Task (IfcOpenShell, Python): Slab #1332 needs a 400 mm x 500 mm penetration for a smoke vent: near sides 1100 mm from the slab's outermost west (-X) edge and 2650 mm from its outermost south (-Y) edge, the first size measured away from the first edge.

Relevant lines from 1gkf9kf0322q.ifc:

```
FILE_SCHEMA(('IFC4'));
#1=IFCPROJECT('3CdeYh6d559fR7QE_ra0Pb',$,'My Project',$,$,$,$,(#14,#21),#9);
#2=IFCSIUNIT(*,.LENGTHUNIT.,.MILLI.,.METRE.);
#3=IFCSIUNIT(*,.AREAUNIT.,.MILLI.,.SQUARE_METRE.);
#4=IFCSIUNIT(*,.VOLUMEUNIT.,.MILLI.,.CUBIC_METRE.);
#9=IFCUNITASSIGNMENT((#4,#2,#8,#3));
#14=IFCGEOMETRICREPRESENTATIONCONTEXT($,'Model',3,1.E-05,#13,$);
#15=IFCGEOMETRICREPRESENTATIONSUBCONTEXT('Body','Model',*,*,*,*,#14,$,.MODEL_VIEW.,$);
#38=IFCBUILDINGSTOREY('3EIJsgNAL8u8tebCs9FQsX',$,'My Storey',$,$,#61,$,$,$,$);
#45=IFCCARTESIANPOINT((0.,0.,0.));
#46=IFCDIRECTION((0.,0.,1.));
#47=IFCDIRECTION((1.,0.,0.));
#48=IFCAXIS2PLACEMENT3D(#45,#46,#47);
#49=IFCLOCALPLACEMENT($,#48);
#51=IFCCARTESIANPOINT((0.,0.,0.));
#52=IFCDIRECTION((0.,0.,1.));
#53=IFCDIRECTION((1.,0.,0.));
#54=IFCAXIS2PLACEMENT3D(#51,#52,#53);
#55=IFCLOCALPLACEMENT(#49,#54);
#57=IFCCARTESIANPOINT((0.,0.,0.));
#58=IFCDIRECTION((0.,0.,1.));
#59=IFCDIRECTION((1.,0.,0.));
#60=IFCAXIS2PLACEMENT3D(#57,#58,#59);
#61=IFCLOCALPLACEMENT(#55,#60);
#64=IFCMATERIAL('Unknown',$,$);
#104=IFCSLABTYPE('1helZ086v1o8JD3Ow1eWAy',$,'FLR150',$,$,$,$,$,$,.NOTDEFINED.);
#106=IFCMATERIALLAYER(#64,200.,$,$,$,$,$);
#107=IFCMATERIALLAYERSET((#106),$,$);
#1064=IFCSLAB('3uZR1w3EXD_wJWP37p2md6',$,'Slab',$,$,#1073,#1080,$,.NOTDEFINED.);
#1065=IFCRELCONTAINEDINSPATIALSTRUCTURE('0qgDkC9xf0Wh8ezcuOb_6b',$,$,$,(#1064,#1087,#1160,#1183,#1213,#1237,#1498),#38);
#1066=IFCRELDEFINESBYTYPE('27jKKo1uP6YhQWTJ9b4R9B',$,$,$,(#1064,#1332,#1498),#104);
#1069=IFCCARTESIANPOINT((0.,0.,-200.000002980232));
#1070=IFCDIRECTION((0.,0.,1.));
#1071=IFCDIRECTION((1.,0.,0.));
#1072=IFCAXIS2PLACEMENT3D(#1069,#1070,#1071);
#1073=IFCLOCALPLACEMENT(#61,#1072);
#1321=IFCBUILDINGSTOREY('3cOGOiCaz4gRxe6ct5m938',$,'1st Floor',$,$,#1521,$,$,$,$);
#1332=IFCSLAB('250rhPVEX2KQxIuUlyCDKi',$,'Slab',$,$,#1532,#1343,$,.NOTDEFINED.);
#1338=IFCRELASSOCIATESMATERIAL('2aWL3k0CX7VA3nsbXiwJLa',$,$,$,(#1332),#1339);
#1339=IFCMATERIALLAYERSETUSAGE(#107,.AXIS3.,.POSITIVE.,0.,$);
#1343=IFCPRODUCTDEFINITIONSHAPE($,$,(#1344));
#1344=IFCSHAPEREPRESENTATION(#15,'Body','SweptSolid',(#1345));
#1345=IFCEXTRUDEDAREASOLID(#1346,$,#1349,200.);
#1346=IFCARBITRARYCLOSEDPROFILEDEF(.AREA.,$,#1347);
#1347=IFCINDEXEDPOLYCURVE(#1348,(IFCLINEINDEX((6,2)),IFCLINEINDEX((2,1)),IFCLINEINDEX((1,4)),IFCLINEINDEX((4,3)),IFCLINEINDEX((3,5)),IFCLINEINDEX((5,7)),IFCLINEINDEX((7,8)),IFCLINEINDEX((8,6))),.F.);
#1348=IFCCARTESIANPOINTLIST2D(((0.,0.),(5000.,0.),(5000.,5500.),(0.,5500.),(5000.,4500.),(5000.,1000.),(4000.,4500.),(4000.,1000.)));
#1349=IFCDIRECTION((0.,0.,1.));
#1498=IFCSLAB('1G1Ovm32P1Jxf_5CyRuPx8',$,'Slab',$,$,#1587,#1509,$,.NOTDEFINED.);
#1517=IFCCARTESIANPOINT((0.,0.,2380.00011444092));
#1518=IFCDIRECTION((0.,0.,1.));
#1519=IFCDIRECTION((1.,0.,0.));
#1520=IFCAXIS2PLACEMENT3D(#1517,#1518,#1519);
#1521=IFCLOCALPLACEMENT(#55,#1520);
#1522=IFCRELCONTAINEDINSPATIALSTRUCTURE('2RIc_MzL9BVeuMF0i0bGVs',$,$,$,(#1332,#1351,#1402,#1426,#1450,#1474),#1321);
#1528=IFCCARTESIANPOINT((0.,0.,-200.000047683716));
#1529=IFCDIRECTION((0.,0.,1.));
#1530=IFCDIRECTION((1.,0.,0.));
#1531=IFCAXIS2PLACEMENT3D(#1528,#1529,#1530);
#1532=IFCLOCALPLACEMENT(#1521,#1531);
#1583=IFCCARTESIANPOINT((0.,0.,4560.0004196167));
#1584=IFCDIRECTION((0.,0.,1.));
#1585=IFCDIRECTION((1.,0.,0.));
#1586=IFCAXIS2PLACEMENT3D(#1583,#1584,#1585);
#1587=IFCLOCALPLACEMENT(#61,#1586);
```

```python
import numpy as np
import ifcopenshell
import ifcopenshell.api.feature
import ifcopenshell.api.geometry
import ifcopenshell.api.root
import ifcopenshell.geom
import ifcopenshell.util.placement
import ifcopenshell.util.representation
import ifcopenshell.util.shape
import ifcopenshell.util.unit

model = ifcopenshell.open("1gkf9kf0322q.ifc")
unit_scale = ifcopenshell.util.unit.calculate_unit_scale(model)
settings = ifcopenshell.geom.settings()


def volume(element):
    """Net volume in cubic metres, openings subtracted."""
    shape = ifcopenshell.geom.create_shape(settings, element)
    return ifcopenshell.util.shape.get_volume(shape.geometry)


slab = model.by_id(1332)
before = volume(slab)

# Extent in the slab's own axes, in metres. The edges named are its -X and -Y sides.
slab_shape = ifcopenshell.geom.create_shape(settings, slab)
vertices = ifcopenshell.util.shape.get_vertices(slab_shape.geometry)
x_min, y_min, bottom = vertices.min(axis=0)
top = vertices[:, 2].max()

opening = ifcopenshell.api.root.create_entity(model, ifc_class="IfcOpeningElement", name="Smoke vent opening", predefined_type="OPENING")
context = ifcopenshell.util.representation.get_context(model, "Model", "Body", "MODEL_VIEW")
width, depth = 0.4, 0.5
outline = [(0.0, 0.0), (width, 0.0), (width, depth), (0.0, depth), (0.0, 0.0)]
# Overshoot both faces by 50 mm so the cut is clean.
shape = ifcopenshell.api.geometry.add_slab_representation(
    model, context=context, depth=top - bottom + 0.1, polyline=outline
)
ifcopenshell.api.geometry.assign_representation(model, product=opening, representation=shape)

matrix = ifcopenshell.util.placement.get_local_placement(slab.ObjectPlacement)
matrix[:, 3] = matrix @ np.append(np.array([x_min + 1.1, y_min + 2.65, bottom - 0.05]) / unit_scale, 1.0)
ifcopenshell.api.geometry.edit_object_placement(model, product=opening, matrix=matrix, is_si=False)
ifcopenshell.api.feature.add_feature(model, feature=opening, element=slab)

after = volume(slab)

print(f"slab volume {before:.3f} -> {after:.3f} m3")

model.write("1gkf9kf0322q_rev.ifc")
```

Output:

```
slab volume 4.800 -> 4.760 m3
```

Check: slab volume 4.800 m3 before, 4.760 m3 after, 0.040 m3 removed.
